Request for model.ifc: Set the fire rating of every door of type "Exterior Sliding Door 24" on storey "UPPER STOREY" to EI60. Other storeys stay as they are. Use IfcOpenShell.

First a look at what the model holds.

```python
import ifcopenshell
import ifcopenshell.util.element

model = ifcopenshell.open("model.ifc")
print(model.schema)
storey = next(s for s in model.by_type("IfcBuildingStorey") if s.Name == "UPPER STOREY")
doors = [e for e in ifcopenshell.util.element.get_decomposition(storey) if e.is_a("IfcDoor")]
seen = {}
for e in doors:
    element_type = ifcopenshell.util.element.get_type(e)
    key = (element_type.Name if element_type != e and element_type else None, ifcopenshell.util.element.get_pset(e, "Pset_DoorCommon", "FireRating"))
    seen[key] = seen.get(key, 0) + 1
for (name, value), count in sorted(seen.items(), key=str):
    print(count, "x", name, "|", value)
```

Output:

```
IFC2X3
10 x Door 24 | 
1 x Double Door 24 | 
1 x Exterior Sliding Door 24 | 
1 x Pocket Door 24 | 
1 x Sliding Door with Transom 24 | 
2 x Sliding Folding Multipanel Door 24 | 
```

```python
import ifcopenshell
import ifcopenshell.api.pset
import ifcopenshell.util.element

model = ifcopenshell.open("model.ifc")

storey = next(s for s in model.by_type("IfcBuildingStorey") if s.Name == "UPPER STOREY")
doors = [e for e in ifcopenshell.util.element.get_decomposition(storey) if e.is_a("IfcDoor")]

count = 0
for e in doors:
    element_type = ifcopenshell.util.element.get_type(e)
    if element_type in (None, e) or element_type.Name != "Exterior Sliding Door 24":
        continue
    # add_pset returns the element's existing set when there is one.
    pset = ifcopenshell.api.pset.add_pset(model, product=e, name="Pset_DoorCommon")
    ifcopenshell.api.pset.edit_pset(model, pset=pset, properties={"FireRating": "EI60"})
    count += 1

print(count, "doors updated")

model.write("model_rev.ifc")
```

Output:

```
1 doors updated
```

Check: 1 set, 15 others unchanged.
